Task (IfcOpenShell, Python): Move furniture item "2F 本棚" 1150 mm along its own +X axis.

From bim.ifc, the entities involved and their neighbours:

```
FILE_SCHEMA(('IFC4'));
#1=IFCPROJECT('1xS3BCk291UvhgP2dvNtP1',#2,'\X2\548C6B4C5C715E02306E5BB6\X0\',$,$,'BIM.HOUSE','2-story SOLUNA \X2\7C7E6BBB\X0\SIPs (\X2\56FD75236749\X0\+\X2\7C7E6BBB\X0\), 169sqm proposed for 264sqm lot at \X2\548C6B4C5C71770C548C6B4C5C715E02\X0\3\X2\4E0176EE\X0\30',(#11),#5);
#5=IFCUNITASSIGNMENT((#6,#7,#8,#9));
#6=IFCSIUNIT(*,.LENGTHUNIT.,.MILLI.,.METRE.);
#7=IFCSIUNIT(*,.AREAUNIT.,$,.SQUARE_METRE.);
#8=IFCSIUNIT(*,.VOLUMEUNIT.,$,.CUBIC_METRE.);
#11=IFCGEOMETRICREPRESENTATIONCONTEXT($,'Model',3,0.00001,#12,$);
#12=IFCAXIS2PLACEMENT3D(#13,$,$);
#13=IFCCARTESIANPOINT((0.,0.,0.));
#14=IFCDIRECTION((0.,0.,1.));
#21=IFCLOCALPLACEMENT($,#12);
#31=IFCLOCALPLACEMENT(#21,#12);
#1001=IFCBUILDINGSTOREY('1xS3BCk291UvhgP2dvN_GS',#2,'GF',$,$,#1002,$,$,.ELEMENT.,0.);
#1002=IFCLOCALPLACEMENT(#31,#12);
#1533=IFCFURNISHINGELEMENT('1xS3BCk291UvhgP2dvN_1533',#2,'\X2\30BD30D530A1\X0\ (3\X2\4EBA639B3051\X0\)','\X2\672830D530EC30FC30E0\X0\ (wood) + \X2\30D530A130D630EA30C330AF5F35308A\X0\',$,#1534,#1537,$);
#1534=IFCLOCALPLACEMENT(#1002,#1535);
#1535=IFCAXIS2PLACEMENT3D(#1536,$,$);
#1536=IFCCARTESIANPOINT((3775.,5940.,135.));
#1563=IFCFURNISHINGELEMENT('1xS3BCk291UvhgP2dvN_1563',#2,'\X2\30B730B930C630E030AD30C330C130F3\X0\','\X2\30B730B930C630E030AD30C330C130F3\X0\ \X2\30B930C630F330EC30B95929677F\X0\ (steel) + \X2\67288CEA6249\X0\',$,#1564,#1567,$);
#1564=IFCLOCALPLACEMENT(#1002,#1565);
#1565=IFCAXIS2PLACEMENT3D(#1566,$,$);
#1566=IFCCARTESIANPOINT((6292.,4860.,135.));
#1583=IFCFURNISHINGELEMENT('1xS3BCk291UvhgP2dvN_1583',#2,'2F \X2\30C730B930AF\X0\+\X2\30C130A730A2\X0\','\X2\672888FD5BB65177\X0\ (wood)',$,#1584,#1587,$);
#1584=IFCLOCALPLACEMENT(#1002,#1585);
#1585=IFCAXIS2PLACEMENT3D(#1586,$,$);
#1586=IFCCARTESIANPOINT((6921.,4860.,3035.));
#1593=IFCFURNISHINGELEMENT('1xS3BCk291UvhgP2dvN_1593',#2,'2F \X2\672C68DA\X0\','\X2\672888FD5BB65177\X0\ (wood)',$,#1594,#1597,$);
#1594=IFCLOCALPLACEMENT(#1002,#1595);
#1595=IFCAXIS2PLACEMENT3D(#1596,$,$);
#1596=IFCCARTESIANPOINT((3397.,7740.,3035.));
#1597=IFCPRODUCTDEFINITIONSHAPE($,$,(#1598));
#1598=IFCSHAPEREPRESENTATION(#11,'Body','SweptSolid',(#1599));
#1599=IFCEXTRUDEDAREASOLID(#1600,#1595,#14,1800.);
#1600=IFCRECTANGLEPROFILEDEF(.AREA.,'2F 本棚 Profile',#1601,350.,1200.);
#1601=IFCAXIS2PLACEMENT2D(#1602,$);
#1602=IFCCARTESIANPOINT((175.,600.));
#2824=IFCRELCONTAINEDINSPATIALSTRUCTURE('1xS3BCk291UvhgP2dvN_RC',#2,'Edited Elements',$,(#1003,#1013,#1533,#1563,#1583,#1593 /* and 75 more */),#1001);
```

```python
import ifcopenshell
import ifcopenshell.api.geometry
import ifcopenshell.util.placement
import ifcopenshell.util.unit

model = ifcopenshell.open("bim.ifc")
unit_scale = ifcopenshell.util.unit.calculate_unit_scale(model)

item = model.by_guid("1xS3BCk291UvhgP2dvN_1593")
matrix = ifcopenshell.util.placement.get_local_placement(item.ObjectPlacement)
matrix[:3, 3] += matrix[:3, 0] * 1.15 / unit_scale
ifcopenshell.api.geometry.edit_object_placement(model, product=item, matrix=matrix, is_si=False)

print(ifcopenshell.util.placement.get_local_placement(item.ObjectPlacement).round(3) + 0.0)

model.write("bim_rev.ifc")
```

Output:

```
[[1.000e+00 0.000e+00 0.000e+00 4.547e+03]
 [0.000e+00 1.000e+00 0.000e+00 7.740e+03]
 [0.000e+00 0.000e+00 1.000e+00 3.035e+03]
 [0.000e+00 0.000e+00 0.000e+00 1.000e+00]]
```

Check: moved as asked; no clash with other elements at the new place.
